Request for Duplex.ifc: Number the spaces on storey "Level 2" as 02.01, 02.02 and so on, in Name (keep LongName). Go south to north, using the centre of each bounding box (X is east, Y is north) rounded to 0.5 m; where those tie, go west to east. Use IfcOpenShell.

First a look at what the model holds.

```python
import ifcopenshell
import ifcopenshell.util.element
import ifcopenshell.util.placement

model = ifcopenshell.open("Duplex.ifc")
print(model.schema)
storey = next(s for s in model.by_type("IfcBuildingStorey") if s.Name == "Level 2")
spaces = [e for e in ifcopenshell.util.element.get_decomposition(storey) if e.is_a("IfcSpace")]
for e in sorted(spaces, key=lambda e: e.id()):
    origin = ifcopenshell.util.placement.get_local_placement(e.ObjectPlacement)[:3, 3]
    print(e.id(), e.Name, e.LongName, origin.round(2) + 0.0, sep=" | ")
```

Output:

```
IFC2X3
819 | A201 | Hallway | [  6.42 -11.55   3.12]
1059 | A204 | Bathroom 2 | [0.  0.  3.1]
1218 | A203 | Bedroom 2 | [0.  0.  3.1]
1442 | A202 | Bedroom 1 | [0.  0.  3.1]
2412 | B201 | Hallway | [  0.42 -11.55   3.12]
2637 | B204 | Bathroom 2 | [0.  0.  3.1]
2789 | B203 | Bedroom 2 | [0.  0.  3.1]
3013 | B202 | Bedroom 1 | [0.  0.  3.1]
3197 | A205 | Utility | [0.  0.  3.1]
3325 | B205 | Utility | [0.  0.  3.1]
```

```python
import ifcopenshell
import ifcopenshell.geom
import ifcopenshell.util.element
import ifcopenshell.util.shape

model = ifcopenshell.open("Duplex.ifc")
settings = ifcopenshell.geom.settings()
settings.set("use-world-coords", True)


def centre(element):
    shape = ifcopenshell.geom.create_shape(settings, element)
    return ifcopenshell.util.shape.get_bbox_centroid(shape.geometry)


storey = next(s for s in model.by_type("IfcBuildingStorey") if s.Name == "Level 2")
spaces = [e for e in ifcopenshell.util.element.get_decomposition(storey) if e.is_a("IfcSpace")]

# Insertion points can sit at a corner or the storey origin, so sort by the geometry (in metres).
centres = {e: centre(e) for e in spaces}
spaces.sort(key=lambda e: (round(centres[e][1] / 0.5), centres[e][0]))

for i, e in enumerate(spaces, start=1):
    number = f"02.{i:02d}"
    e.Name = number
    print(e.id(), number)

model.write("Duplex_rev.ifc")
```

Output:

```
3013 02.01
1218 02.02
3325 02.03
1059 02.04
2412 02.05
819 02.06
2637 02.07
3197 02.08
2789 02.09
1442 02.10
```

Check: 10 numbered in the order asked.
